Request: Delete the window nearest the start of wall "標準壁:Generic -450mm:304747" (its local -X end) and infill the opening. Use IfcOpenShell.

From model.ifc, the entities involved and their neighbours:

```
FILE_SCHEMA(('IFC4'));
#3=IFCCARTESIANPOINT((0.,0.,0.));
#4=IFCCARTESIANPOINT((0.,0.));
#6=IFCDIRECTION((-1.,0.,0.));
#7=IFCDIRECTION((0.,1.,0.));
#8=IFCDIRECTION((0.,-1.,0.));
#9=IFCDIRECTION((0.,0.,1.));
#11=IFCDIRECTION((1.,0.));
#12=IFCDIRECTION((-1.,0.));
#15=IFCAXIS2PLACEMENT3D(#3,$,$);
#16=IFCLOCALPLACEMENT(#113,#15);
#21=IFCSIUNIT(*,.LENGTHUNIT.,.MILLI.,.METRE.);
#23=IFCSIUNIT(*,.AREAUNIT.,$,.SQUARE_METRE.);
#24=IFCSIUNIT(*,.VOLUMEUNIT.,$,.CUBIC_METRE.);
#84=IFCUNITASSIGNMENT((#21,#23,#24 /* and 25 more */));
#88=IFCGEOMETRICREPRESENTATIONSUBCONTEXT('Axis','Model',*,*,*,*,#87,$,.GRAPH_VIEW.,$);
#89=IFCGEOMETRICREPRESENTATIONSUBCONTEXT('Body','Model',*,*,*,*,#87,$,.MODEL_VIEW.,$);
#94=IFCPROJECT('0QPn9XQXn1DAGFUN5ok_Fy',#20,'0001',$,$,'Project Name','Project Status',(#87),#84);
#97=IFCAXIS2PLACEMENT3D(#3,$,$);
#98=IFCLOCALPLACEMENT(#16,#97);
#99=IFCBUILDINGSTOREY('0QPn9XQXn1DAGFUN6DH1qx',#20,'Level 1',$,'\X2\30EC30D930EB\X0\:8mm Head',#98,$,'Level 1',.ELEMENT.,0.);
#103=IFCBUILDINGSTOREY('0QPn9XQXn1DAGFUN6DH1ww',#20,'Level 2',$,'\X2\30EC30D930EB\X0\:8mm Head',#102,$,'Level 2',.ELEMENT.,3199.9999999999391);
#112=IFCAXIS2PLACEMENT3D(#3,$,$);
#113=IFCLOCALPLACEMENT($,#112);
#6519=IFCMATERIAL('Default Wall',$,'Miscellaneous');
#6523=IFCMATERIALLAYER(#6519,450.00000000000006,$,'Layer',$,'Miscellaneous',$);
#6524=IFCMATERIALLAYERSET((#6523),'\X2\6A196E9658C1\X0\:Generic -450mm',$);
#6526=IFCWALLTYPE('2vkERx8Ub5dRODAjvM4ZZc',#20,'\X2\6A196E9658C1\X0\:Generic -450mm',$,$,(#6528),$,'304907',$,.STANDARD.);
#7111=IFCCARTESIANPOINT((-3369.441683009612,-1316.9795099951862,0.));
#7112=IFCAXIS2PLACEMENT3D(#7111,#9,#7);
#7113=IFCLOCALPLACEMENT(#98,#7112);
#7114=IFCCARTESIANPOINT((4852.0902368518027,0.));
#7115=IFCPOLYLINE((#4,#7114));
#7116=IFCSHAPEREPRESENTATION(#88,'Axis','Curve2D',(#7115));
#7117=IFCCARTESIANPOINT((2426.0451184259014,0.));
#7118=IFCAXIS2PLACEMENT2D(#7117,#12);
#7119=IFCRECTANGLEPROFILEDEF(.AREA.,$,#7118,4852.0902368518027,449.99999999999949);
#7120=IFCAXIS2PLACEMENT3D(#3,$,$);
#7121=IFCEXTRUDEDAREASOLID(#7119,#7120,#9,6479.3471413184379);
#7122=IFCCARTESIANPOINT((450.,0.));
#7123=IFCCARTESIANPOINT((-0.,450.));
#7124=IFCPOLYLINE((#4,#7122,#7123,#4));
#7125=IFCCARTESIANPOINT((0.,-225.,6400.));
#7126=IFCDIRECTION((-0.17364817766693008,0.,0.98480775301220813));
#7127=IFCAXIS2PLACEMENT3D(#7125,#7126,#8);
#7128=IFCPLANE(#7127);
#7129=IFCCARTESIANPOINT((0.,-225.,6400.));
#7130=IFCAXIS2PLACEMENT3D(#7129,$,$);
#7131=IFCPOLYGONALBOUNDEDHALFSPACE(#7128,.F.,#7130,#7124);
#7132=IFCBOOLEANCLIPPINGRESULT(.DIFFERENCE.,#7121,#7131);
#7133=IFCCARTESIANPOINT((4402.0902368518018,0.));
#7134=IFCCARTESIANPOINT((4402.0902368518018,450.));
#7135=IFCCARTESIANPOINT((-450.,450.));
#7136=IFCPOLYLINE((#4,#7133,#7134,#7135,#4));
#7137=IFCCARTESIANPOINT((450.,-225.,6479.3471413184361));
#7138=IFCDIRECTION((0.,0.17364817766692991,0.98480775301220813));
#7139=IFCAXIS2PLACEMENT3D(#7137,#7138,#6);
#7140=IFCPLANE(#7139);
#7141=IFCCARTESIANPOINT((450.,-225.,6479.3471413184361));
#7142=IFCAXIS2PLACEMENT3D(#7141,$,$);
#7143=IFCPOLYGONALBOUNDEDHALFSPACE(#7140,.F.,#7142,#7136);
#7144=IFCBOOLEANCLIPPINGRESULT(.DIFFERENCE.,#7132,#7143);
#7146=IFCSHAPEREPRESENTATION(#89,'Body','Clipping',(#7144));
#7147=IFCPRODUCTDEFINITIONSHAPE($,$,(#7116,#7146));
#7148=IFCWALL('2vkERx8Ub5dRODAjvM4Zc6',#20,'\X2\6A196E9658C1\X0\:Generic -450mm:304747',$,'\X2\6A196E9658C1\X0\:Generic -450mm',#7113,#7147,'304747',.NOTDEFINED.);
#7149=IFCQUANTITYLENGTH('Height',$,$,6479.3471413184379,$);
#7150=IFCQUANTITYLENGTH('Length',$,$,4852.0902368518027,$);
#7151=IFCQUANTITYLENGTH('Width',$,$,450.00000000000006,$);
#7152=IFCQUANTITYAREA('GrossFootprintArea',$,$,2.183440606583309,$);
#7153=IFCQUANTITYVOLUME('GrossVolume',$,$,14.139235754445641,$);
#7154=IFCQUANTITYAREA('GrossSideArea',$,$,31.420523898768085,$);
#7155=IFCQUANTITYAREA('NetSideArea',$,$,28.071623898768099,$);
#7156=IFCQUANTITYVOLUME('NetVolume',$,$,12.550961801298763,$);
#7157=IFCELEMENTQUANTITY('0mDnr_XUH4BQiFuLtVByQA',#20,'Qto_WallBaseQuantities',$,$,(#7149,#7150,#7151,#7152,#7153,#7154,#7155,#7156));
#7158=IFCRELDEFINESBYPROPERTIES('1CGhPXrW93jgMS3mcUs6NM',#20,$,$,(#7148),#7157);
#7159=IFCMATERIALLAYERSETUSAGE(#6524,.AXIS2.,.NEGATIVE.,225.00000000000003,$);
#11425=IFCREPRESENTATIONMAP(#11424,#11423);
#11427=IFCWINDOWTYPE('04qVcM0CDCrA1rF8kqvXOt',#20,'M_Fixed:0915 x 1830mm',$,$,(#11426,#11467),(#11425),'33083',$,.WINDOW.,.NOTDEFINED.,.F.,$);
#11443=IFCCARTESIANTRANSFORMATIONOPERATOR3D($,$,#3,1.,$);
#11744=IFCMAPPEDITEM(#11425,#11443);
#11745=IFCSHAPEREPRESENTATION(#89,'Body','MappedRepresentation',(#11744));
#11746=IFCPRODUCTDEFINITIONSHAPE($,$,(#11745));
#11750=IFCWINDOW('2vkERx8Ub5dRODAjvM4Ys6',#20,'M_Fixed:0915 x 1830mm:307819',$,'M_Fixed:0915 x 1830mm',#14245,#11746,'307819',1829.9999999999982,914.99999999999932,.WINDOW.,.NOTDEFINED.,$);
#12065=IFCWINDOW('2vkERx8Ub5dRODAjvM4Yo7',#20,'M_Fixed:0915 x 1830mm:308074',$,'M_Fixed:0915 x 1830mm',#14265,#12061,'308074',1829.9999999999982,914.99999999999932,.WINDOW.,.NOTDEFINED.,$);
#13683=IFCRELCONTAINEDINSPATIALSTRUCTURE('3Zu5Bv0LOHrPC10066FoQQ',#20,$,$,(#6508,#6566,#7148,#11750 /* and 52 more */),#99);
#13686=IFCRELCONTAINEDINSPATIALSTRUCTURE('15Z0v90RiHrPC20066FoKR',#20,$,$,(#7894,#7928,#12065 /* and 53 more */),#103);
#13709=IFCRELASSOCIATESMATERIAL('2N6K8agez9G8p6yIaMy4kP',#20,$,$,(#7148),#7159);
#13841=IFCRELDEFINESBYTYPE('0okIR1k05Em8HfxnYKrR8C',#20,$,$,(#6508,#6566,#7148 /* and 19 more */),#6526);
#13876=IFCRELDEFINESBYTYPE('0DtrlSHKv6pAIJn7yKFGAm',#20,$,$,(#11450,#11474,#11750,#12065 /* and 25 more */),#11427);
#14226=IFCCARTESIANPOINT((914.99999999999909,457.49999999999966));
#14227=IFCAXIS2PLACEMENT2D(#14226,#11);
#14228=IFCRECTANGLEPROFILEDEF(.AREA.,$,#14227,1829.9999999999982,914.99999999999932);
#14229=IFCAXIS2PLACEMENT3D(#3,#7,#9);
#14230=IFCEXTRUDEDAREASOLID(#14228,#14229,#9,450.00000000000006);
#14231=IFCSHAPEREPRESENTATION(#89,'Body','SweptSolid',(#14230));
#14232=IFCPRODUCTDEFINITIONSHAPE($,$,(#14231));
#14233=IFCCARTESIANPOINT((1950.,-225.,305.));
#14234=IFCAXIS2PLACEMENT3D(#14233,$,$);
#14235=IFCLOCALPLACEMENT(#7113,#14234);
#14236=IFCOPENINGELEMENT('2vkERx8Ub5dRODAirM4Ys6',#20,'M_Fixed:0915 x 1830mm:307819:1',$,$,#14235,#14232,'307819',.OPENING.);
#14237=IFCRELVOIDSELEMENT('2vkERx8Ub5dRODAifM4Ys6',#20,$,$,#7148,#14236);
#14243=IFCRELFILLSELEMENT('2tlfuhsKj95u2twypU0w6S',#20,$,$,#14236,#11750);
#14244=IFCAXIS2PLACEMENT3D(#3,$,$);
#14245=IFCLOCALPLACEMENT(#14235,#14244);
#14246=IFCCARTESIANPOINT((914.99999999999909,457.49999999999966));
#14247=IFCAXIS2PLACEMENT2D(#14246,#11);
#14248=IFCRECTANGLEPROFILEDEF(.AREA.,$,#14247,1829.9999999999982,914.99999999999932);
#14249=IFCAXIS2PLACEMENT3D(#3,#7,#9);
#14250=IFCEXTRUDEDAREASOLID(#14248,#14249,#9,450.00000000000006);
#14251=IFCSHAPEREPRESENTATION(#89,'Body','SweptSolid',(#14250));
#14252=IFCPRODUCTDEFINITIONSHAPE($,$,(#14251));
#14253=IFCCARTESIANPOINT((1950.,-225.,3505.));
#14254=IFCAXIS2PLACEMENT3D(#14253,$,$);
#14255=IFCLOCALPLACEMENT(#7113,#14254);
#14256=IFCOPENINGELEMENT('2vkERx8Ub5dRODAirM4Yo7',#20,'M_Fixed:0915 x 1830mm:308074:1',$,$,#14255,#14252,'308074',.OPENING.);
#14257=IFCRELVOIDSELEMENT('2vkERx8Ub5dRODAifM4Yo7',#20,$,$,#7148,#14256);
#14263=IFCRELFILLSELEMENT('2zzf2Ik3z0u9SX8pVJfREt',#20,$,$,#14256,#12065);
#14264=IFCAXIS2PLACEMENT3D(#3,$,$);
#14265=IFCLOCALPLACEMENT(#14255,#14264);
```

```python
import ifcopenshell
import ifcopenshell.api.feature
import ifcopenshell.api.pset
import ifcopenshell.api.root
import ifcopenshell.geom
import ifcopenshell.util.element
import ifcopenshell.util.shape
import ifcopenshell.util.unit

model = ifcopenshell.open("model.ifc")
area_scale = ifcopenshell.util.unit.calculate_unit_scale(model, "AREAUNIT")
volume_scale = ifcopenshell.util.unit.calculate_unit_scale(model, "VOLUMEUNIT")
settings = ifcopenshell.geom.settings()


def volume(element):
    """Net volume in cubic metres, openings subtracted."""
    shape = ifcopenshell.geom.create_shape(settings, element)
    return ifcopenshell.util.shape.get_volume(shape.geometry)


window = model.by_guid("2vkERx8Ub5dRODAjvM4Ys6")
opening = window.FillsVoids[0].RelatingOpeningElement
wall = opening.VoidsElements[0].RelatingBuildingElement
before = volume(wall)

ifcopenshell.api.root.remove_product(model, product=window)
ifcopenshell.api.feature.remove_feature(model, feature=opening)

after = volume(wall)
thickness = 0.45  # wall thickness in metres

# Update the wall's stored quantities.
qto = model.by_id(ifcopenshell.util.element.get_pset(wall, "Qto_WallBaseQuantities", should_inherit=False)["id"])
ifcopenshell.api.pset.edit_qto(model, qto=qto, properties={
    "NetSideArea": after / thickness / area_scale,
    "NetVolume": after / volume_scale,
})

print(f"wall volume {before:.3f} -> {after:.3f} m3")

model.write("model_rev.ifc")
```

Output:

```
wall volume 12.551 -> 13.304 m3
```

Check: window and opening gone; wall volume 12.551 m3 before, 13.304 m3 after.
